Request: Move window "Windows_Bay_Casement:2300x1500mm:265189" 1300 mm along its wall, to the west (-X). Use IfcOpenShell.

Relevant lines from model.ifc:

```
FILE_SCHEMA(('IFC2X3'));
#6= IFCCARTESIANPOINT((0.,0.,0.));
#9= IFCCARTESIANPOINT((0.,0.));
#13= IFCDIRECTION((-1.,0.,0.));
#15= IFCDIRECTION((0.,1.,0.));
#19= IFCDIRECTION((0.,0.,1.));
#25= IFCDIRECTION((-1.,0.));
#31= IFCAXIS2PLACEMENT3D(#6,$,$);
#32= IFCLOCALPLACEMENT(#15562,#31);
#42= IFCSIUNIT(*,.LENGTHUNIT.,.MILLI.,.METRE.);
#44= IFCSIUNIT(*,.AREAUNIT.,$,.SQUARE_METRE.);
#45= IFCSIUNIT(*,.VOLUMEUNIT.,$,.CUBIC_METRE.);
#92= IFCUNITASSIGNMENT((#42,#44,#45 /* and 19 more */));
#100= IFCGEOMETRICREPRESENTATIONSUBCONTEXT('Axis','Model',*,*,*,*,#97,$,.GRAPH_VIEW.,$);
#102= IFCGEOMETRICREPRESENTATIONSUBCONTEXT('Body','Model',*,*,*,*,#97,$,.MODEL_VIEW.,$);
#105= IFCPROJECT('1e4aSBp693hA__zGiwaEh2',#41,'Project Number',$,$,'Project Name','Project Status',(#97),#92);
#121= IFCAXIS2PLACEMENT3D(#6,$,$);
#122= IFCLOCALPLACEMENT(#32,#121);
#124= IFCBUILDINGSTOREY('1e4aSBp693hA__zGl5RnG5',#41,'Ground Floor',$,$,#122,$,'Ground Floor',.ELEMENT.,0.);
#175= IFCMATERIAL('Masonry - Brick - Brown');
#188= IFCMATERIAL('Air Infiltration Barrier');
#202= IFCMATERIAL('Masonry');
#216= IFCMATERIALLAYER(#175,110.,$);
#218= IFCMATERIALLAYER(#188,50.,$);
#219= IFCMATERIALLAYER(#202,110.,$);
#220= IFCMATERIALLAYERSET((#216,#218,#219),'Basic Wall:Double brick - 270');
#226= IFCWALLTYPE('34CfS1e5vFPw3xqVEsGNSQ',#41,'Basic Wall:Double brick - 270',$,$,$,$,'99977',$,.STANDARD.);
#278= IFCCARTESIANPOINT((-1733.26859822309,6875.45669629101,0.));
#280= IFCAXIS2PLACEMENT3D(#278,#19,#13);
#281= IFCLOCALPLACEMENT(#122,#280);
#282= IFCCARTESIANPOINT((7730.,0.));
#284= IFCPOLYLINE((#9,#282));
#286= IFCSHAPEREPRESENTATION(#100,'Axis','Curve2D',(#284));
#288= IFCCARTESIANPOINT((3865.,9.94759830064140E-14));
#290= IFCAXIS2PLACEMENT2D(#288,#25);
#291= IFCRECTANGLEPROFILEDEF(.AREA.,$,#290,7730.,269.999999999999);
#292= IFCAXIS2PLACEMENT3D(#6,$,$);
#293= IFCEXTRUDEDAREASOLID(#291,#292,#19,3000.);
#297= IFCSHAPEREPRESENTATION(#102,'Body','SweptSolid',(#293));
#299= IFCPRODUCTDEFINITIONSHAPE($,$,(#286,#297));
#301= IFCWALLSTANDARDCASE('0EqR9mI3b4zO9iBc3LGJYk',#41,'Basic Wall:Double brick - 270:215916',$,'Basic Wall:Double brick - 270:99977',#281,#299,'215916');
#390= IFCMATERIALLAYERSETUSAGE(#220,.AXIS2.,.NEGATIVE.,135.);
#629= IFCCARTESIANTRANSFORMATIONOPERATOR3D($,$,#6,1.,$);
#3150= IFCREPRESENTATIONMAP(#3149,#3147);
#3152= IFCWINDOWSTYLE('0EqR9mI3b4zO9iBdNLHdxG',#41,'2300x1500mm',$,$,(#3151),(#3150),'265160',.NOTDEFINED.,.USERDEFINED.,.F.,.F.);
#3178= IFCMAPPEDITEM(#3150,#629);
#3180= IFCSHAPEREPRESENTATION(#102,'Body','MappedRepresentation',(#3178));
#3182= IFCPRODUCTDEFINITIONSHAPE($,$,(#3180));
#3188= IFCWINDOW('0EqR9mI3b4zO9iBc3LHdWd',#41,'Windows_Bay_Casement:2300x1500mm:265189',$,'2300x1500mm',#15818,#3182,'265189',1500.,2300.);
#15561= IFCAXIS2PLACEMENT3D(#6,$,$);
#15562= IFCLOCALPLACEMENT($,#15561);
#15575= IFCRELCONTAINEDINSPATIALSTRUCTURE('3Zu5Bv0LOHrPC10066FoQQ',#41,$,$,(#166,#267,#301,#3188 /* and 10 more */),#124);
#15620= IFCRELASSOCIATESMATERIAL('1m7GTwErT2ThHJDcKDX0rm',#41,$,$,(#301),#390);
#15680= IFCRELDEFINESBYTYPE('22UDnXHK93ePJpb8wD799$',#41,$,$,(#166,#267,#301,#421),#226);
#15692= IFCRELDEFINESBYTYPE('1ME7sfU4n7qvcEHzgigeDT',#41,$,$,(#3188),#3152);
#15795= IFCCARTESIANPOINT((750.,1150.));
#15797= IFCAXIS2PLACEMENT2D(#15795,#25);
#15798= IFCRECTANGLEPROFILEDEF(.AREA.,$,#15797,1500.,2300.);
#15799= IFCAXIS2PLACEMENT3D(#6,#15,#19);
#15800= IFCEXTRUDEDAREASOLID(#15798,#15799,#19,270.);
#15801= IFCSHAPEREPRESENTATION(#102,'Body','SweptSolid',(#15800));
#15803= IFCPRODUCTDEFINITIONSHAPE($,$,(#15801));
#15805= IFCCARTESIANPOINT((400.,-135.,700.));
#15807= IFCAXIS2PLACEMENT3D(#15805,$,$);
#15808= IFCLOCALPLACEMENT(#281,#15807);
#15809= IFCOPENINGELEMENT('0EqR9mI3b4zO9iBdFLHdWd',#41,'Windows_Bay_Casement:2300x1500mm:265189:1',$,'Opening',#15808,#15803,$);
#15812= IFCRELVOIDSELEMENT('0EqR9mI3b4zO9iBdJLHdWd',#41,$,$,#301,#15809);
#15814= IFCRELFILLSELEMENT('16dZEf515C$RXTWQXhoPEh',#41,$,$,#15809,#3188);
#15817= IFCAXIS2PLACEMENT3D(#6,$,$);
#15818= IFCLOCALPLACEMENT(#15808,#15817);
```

```python
import ifcopenshell
import ifcopenshell.api.geometry
import ifcopenshell.util.placement
import ifcopenshell.util.unit

model = ifcopenshell.open("model.ifc")
unit_scale = ifcopenshell.util.unit.calculate_unit_scale(model)

window = model.by_guid("0EqR9mI3b4zO9iBc3LHdWd")
opening = window.FillsVoids[0].RelatingOpeningElement
wall = opening.VoidsElements[0].RelatingBuildingElement

wall_matrix = ifcopenshell.util.placement.get_local_placement(wall.ObjectPlacement)
shift = wall_matrix[:3, 0] * 1.3 / unit_scale
before = ifcopenshell.util.placement.get_local_placement(window.ObjectPlacement)[:3, 3].copy()

# The window is placed relative to its opening, so it follows when the opening moves.
matrix = ifcopenshell.util.placement.get_local_placement(opening.ObjectPlacement)
matrix[:3, 3] += shift
ifcopenshell.api.geometry.edit_object_placement(
    model, product=opening, matrix=matrix, is_si=False, should_transform_children=True
)

after = ifcopenshell.util.placement.get_local_placement(window.ObjectPlacement)[:3, 3]
print("window moved by", (after - before).round(3) + 0.0)

model.write("model_rev.ifc")
```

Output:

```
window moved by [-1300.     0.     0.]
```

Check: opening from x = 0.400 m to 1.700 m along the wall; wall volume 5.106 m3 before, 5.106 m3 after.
